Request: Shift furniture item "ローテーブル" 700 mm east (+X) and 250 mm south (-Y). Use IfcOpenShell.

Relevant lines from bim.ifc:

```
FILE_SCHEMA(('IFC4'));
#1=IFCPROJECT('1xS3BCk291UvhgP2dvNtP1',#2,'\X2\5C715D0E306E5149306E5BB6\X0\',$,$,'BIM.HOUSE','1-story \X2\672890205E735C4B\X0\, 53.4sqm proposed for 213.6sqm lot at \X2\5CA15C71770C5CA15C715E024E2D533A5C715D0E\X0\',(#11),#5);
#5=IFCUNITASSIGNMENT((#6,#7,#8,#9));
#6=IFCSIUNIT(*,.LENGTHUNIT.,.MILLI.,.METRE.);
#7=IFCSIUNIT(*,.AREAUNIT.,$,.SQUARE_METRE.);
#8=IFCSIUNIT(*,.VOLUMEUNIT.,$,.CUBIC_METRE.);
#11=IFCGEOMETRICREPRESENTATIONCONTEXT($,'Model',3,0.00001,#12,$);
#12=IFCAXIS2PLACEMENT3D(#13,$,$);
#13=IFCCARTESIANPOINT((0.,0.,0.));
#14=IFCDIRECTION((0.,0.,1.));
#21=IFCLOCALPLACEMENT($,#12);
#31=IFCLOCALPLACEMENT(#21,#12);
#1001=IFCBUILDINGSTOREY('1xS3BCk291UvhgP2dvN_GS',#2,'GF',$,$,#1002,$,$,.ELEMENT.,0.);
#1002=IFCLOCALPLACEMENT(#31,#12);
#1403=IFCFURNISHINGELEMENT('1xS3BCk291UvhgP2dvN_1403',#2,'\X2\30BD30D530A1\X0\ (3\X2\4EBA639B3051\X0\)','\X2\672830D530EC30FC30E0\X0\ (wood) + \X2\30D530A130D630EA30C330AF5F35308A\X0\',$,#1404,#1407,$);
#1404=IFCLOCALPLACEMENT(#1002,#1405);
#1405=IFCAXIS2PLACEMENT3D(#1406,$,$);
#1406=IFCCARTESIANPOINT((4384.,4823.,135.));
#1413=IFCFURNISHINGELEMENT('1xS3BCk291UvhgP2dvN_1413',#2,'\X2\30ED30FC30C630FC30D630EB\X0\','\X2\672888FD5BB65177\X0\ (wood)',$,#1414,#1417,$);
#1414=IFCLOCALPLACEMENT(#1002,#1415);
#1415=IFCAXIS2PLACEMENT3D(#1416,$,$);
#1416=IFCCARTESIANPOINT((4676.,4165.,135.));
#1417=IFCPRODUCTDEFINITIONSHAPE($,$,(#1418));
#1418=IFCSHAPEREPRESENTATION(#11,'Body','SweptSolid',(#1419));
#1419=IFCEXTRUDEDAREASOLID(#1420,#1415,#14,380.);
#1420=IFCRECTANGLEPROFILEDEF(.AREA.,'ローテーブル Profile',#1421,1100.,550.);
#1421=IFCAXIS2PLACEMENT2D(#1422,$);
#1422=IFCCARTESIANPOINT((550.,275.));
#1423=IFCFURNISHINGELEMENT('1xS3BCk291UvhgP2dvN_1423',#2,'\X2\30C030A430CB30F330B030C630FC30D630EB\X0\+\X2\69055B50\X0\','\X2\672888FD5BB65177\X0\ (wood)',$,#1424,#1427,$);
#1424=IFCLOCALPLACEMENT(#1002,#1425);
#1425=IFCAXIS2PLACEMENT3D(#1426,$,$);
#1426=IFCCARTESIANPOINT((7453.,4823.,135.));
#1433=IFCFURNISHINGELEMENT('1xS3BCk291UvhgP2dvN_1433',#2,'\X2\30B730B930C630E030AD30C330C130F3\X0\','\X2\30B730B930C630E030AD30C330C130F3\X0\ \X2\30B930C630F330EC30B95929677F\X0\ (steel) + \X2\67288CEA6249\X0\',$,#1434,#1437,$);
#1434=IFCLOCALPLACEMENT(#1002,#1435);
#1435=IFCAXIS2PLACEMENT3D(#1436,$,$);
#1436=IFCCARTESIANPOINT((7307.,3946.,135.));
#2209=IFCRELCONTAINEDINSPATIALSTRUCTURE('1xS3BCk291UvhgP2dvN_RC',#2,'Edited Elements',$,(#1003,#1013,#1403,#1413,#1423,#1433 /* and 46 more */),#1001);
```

```python
import ifcopenshell
import ifcopenshell.api.geometry
import ifcopenshell.util.placement
import ifcopenshell.util.unit

model = ifcopenshell.open("bim.ifc")
unit_scale = ifcopenshell.util.unit.calculate_unit_scale(model)

item = model.by_guid("1xS3BCk291UvhgP2dvN_1413")
matrix = ifcopenshell.util.placement.get_local_placement(item.ObjectPlacement)
matrix[0, 3] += 0.7 / unit_scale
matrix[1, 3] -= 0.25 / unit_scale
ifcopenshell.api.geometry.edit_object_placement(model, product=item, matrix=matrix, is_si=False)

print(ifcopenshell.util.placement.get_local_placement(item.ObjectPlacement).round(3) + 0.0)

model.write("bim_rev.ifc")
```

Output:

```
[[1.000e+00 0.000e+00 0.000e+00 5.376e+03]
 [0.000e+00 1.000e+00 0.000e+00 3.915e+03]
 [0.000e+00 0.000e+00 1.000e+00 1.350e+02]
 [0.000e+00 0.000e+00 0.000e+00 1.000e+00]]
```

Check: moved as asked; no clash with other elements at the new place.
